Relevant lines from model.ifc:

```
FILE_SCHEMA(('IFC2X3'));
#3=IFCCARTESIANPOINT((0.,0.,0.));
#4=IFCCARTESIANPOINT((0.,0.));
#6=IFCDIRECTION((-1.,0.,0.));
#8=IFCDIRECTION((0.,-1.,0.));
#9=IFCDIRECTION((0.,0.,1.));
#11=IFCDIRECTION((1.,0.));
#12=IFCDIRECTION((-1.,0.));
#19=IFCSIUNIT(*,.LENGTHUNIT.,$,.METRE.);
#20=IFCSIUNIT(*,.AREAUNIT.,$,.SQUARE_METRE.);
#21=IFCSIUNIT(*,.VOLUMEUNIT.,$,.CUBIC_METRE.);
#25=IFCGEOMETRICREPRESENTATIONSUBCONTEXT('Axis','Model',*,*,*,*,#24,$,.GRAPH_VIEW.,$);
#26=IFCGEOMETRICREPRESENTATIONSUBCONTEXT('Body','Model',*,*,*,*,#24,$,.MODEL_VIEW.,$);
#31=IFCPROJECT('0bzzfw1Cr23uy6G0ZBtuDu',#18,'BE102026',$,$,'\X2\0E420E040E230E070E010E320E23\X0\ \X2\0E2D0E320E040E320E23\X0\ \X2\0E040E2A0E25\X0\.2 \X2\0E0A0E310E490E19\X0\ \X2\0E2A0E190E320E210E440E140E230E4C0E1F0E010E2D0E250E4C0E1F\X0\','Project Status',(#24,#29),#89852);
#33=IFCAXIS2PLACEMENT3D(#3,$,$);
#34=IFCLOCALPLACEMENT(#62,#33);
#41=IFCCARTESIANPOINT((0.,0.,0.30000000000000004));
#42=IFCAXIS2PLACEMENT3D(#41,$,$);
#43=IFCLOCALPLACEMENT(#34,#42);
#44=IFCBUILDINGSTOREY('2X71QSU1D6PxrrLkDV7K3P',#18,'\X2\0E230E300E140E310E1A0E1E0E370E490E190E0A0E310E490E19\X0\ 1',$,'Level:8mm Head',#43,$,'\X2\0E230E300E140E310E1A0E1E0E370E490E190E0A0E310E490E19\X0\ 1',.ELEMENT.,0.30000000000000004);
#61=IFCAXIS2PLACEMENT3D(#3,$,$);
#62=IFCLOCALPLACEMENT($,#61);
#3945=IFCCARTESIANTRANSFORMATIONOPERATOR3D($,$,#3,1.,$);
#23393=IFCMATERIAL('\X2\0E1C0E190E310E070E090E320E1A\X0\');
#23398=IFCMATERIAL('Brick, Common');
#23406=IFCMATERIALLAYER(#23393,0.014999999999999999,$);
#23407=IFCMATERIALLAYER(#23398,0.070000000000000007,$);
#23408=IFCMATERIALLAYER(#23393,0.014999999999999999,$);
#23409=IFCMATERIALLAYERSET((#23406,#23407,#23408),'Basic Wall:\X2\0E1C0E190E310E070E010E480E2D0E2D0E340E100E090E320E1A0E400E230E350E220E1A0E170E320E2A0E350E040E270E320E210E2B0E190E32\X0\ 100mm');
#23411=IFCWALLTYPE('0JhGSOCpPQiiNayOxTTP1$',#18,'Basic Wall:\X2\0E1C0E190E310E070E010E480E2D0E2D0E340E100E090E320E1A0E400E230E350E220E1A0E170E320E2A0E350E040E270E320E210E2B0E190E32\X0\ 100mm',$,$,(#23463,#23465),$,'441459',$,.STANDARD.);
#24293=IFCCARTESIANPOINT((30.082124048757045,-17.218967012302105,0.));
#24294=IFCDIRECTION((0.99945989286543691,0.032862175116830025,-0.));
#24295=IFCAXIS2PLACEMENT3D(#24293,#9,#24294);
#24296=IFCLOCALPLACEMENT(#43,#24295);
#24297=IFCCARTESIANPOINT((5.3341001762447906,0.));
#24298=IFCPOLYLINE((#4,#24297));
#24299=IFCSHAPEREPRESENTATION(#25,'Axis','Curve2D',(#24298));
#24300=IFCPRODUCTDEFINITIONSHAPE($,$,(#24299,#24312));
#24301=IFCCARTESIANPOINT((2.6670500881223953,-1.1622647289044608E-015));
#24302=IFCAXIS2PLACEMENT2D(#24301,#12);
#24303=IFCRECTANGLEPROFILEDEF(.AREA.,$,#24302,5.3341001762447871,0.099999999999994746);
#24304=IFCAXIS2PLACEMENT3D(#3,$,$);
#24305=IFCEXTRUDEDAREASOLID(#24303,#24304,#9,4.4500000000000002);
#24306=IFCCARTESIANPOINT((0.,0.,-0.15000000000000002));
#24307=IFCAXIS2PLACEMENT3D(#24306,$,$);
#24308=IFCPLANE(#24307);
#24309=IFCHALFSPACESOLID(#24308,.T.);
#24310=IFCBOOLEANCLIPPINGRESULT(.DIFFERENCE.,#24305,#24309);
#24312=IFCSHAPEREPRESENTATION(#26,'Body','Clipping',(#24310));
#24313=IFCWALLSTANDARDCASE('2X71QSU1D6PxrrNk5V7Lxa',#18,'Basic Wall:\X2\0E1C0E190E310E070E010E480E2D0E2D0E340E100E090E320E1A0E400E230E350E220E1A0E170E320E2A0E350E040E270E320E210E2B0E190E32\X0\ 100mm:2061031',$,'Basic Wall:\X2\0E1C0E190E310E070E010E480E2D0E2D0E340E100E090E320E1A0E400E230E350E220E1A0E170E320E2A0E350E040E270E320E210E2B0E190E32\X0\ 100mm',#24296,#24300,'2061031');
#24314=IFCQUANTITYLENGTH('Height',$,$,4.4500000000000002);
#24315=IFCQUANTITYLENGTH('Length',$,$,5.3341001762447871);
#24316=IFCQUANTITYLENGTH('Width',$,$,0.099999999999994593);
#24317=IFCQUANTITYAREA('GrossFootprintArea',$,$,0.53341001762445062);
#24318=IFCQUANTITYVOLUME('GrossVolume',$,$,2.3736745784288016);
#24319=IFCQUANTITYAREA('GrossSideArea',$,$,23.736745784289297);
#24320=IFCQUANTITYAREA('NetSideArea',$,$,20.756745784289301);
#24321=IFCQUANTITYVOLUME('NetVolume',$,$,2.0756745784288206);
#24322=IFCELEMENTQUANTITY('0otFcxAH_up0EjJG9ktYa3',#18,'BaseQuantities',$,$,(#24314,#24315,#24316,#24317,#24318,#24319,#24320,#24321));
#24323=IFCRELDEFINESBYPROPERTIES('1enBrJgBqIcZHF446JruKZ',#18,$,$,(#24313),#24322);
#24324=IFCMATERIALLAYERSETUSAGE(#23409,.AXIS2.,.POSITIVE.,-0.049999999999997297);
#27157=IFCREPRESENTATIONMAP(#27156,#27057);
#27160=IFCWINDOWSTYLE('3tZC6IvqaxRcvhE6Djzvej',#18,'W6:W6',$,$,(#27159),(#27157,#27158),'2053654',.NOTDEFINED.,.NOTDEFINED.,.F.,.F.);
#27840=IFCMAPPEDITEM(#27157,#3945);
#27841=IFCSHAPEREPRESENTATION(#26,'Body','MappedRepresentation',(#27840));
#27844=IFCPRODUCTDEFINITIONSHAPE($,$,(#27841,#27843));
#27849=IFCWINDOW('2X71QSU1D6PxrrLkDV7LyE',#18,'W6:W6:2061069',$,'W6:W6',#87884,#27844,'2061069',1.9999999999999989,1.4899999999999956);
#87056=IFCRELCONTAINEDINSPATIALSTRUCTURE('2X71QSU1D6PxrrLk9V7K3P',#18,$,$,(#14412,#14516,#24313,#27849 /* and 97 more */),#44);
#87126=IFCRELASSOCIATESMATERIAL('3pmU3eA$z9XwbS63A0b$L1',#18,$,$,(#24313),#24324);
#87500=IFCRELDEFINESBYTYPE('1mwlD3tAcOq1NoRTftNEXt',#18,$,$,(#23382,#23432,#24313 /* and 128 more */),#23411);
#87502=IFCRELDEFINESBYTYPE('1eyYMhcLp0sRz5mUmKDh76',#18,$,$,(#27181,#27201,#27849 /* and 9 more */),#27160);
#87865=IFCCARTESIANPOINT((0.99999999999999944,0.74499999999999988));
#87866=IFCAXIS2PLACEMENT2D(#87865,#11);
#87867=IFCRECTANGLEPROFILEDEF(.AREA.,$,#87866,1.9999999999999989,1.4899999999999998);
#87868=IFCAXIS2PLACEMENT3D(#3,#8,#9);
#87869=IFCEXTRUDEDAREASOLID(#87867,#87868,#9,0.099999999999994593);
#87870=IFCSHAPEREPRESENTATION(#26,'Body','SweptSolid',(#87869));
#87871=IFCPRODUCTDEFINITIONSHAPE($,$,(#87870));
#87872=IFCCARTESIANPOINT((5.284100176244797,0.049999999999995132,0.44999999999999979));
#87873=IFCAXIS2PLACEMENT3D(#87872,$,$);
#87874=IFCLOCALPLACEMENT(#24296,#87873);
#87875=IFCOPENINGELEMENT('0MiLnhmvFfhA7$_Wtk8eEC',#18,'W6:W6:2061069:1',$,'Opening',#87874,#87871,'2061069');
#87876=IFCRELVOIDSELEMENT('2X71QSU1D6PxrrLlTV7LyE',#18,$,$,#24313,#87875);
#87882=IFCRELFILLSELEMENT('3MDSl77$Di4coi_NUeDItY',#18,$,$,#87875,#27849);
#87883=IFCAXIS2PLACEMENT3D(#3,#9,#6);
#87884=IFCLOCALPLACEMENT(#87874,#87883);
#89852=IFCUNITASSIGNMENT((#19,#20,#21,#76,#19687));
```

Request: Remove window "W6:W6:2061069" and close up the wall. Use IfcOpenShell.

```python
import ifcopenshell
import ifcopenshell.api.feature
import ifcopenshell.api.pset
import ifcopenshell.api.root
import ifcopenshell.geom
import ifcopenshell.util.element
import ifcopenshell.util.shape
import ifcopenshell.util.unit

model = ifcopenshell.open("model.ifc")
area_scale = ifcopenshell.util.unit.calculate_unit_scale(model, "AREAUNIT")
volume_scale = ifcopenshell.util.unit.calculate_unit_scale(model, "VOLUMEUNIT")
settings = ifcopenshell.geom.settings()


def volume(element):
    """Net volume in cubic metres, openings subtracted."""
    shape = ifcopenshell.geom.create_shape(settings, element)
    return ifcopenshell.util.shape.get_volume(shape.geometry)


window = model.by_guid("2X71QSU1D6PxrrLkDV7LyE")
opening = window.FillsVoids[0].RelatingOpeningElement
wall = opening.VoidsElements[0].RelatingBuildingElement
before = volume(wall)

ifcopenshell.api.root.remove_product(model, product=window)
ifcopenshell.api.feature.remove_feature(model, feature=opening)

after = volume(wall)
thickness = 0.1  # wall thickness in metres

# Update the wall's stored quantities.
qto = model.by_id(ifcopenshell.util.element.get_pset(wall, "BaseQuantities", should_inherit=False)["id"])
ifcopenshell.api.pset.edit_qto(model, qto=qto, properties={
    "NetSideArea": after / thickness / area_scale,
    "NetVolume": after / volume_scale,
})

print(f"wall volume {before:.3f} -> {after:.3f} m3")

model.write("model_v2.ifc")
```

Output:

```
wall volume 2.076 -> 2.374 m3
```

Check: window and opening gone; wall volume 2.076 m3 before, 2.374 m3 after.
